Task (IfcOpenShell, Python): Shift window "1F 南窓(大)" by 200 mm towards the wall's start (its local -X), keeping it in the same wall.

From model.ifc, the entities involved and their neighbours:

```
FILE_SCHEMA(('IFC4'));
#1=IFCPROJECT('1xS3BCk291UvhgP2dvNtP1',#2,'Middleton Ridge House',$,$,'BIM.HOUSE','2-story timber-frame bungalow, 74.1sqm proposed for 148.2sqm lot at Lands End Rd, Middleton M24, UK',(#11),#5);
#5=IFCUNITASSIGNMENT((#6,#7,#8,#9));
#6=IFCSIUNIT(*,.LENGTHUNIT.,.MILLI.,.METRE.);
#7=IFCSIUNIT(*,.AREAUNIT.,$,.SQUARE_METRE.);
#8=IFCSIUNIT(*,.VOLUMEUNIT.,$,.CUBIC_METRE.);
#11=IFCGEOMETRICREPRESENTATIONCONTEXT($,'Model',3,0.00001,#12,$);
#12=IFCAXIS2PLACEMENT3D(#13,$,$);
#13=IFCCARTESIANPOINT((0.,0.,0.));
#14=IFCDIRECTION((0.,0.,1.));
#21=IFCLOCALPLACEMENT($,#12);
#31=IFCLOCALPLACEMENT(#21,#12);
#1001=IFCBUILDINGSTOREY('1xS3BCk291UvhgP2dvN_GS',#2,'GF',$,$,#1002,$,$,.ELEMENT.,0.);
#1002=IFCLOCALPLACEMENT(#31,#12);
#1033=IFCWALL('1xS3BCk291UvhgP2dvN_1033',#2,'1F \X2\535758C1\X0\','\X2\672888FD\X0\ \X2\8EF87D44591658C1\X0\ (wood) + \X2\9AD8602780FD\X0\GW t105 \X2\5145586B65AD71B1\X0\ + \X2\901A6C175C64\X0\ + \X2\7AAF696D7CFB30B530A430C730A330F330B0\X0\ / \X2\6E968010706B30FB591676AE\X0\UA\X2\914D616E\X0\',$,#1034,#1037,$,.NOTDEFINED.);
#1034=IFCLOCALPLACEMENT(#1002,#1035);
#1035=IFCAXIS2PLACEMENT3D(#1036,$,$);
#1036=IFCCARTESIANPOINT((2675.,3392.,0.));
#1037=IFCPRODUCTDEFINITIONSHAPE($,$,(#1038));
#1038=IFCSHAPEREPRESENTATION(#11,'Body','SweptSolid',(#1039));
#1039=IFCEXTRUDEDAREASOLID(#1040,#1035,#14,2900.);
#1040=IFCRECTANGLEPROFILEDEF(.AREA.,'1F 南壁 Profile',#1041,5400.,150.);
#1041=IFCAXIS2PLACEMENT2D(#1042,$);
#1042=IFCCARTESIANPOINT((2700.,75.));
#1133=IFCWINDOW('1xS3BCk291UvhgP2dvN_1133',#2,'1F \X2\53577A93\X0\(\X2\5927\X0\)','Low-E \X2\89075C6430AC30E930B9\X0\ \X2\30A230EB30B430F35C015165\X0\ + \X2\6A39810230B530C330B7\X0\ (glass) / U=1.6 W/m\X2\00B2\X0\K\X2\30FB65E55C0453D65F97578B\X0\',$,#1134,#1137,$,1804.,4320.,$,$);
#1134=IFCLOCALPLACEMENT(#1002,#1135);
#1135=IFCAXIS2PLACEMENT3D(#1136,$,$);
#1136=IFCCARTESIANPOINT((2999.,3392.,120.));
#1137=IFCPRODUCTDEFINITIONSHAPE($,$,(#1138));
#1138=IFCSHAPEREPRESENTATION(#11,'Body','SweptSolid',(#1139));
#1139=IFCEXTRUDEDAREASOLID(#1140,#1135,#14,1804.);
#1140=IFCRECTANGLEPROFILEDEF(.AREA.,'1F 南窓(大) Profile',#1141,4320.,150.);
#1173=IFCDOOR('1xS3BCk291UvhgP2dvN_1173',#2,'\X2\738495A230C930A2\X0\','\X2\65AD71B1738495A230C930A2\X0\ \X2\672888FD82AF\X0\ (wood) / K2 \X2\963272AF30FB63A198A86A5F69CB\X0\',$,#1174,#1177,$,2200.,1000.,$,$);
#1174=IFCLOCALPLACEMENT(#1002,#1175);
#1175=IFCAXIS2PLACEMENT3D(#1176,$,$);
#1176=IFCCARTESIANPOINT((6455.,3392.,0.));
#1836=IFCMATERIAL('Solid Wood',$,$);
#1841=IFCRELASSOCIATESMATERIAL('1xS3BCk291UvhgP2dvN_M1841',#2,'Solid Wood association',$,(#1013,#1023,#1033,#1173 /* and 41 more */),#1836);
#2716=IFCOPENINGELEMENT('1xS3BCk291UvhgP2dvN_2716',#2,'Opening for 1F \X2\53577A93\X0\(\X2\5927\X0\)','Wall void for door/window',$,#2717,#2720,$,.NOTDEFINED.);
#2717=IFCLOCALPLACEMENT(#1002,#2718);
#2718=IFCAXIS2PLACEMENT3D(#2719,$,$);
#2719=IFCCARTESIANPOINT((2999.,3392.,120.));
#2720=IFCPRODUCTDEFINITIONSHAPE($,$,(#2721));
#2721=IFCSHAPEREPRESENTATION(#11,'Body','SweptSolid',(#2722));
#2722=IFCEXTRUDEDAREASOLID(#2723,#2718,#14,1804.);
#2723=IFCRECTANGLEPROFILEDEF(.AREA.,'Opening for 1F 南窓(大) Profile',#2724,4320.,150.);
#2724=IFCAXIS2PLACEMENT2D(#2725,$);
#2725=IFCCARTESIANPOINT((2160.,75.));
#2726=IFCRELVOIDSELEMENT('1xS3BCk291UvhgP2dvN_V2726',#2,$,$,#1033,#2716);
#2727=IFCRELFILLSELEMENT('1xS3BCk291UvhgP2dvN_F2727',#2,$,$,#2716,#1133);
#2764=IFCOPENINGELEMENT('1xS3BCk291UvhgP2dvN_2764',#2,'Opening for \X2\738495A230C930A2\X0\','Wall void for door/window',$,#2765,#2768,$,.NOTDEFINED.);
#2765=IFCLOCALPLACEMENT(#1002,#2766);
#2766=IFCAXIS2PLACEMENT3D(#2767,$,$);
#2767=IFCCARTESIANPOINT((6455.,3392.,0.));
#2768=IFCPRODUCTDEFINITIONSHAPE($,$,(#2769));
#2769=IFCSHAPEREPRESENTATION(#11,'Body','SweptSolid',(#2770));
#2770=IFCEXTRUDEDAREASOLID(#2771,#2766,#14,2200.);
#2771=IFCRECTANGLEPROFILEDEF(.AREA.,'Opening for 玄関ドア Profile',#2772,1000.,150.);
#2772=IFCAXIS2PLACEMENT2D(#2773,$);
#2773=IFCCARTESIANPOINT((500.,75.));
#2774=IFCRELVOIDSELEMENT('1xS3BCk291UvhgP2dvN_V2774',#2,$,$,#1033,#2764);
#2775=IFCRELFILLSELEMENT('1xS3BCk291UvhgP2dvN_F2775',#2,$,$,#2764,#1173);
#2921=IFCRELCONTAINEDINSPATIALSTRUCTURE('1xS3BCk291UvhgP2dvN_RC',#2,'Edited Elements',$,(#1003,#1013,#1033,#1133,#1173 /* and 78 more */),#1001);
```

```python
import ifcopenshell
import ifcopenshell.api.geometry
import ifcopenshell.util.placement
import ifcopenshell.util.unit

model = ifcopenshell.open("model.ifc")
unit_scale = ifcopenshell.util.unit.calculate_unit_scale(model)

window = model.by_guid("1xS3BCk291UvhgP2dvN_1133")
opening = window.FillsVoids[0].RelatingOpeningElement
wall = opening.VoidsElements[0].RelatingBuildingElement

wall_matrix = ifcopenshell.util.placement.get_local_placement(wall.ObjectPlacement)
shift = wall_matrix[:3, 0] * -0.2 / unit_scale
before = ifcopenshell.util.placement.get_local_placement(window.ObjectPlacement)[:3, 3].copy()

# The window is not placed relative to its opening, so move both.
for product in (opening, window):
    matrix = ifcopenshell.util.placement.get_local_placement(product.ObjectPlacement)
    matrix[:3, 3] += shift
    ifcopenshell.api.geometry.edit_object_placement(model, product=product, matrix=matrix, is_si=False)

after = ifcopenshell.util.placement.get_local_placement(window.ObjectPlacement)[:3, 3]
print("window moved by", (after - before).round(3) + 0.0)

model.write("model-out.ifc")
```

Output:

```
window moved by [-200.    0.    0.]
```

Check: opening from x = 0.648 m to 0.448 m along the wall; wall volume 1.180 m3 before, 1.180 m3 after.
